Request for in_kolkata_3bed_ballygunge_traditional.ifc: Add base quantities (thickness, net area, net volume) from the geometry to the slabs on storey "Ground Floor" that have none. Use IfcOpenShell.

First a look at what the model holds.

```python
import ifcopenshell
import ifcopenshell.util.element
import ifcopenshell.util.unit

model = ifcopenshell.open("in_kolkata_3bed_ballygunge_traditional.ifc")
print(model.schema)
for unit_type in ("LENGTHUNIT", "AREAUNIT", "VOLUMEUNIT"):
    print(unit_type, ifcopenshell.util.unit.calculate_unit_scale(model, unit_type))
storey = next(s for s in model.by_type("IfcBuildingStorey") if s.Name == "Ground Floor")
slabs = [e for e in ifcopenshell.util.element.get_decomposition(storey) if e.is_a("IfcSlab")]
for e in sorted(slabs, key=lambda e: e.id()):
    print(e.id(), e.is_a(), e.Name, list(ifcopenshell.util.element.get_psets(e, qtos_only=True)), sep=" | ")
```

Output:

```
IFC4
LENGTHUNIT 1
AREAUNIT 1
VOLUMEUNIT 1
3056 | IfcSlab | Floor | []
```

```python
import ifcopenshell
import ifcopenshell.api.pset
import ifcopenshell.geom
import ifcopenshell.util.element
import ifcopenshell.util.shape
import ifcopenshell.util.unit

model = ifcopenshell.open("in_kolkata_3bed_ballygunge_traditional.ifc")
unit_scale = ifcopenshell.util.unit.calculate_unit_scale(model)
area_scale = ifcopenshell.util.unit.calculate_unit_scale(model, "AREAUNIT")
volume_scale = ifcopenshell.util.unit.calculate_unit_scale(model, "VOLUMEUNIT")
settings = ifcopenshell.geom.settings()

storey = next(s for s in model.by_type("IfcBuildingStorey") if s.Name == "Ground Floor")
slabs = [e for e in ifcopenshell.util.element.get_decomposition(storey) if e.is_a("IfcSlab")]

for e in sorted(slabs, key=lambda e: e.id()):
    if ifcopenshell.util.element.get_psets(e, qtos_only=True, should_inherit=False):
        continue
    # Geometry comes back in metres, in the element's own axes.
    shape = ifcopenshell.geom.create_shape(settings, e)
    values = {
        "Width": ifcopenshell.util.shape.get_z(shape.geometry) / unit_scale,
        "NetArea": ifcopenshell.util.shape.get_footprint_area(shape.geometry) / area_scale,
        "NetVolume": ifcopenshell.util.shape.get_volume(shape.geometry) / volume_scale,
    }
    qto = ifcopenshell.api.pset.add_qto(model, product=e, name="Qto_SlabBaseQuantities")
    ifcopenshell.api.pset.edit_qto(model, qto=qto, properties=values)
    print(e.id(), {k: round(v, 3) for k, v in values.items()})

model.write("in_kolkata_3bed_ballygunge_traditional_rev.ifc")
```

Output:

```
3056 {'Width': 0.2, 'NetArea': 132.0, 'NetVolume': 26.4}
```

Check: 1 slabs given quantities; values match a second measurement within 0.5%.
